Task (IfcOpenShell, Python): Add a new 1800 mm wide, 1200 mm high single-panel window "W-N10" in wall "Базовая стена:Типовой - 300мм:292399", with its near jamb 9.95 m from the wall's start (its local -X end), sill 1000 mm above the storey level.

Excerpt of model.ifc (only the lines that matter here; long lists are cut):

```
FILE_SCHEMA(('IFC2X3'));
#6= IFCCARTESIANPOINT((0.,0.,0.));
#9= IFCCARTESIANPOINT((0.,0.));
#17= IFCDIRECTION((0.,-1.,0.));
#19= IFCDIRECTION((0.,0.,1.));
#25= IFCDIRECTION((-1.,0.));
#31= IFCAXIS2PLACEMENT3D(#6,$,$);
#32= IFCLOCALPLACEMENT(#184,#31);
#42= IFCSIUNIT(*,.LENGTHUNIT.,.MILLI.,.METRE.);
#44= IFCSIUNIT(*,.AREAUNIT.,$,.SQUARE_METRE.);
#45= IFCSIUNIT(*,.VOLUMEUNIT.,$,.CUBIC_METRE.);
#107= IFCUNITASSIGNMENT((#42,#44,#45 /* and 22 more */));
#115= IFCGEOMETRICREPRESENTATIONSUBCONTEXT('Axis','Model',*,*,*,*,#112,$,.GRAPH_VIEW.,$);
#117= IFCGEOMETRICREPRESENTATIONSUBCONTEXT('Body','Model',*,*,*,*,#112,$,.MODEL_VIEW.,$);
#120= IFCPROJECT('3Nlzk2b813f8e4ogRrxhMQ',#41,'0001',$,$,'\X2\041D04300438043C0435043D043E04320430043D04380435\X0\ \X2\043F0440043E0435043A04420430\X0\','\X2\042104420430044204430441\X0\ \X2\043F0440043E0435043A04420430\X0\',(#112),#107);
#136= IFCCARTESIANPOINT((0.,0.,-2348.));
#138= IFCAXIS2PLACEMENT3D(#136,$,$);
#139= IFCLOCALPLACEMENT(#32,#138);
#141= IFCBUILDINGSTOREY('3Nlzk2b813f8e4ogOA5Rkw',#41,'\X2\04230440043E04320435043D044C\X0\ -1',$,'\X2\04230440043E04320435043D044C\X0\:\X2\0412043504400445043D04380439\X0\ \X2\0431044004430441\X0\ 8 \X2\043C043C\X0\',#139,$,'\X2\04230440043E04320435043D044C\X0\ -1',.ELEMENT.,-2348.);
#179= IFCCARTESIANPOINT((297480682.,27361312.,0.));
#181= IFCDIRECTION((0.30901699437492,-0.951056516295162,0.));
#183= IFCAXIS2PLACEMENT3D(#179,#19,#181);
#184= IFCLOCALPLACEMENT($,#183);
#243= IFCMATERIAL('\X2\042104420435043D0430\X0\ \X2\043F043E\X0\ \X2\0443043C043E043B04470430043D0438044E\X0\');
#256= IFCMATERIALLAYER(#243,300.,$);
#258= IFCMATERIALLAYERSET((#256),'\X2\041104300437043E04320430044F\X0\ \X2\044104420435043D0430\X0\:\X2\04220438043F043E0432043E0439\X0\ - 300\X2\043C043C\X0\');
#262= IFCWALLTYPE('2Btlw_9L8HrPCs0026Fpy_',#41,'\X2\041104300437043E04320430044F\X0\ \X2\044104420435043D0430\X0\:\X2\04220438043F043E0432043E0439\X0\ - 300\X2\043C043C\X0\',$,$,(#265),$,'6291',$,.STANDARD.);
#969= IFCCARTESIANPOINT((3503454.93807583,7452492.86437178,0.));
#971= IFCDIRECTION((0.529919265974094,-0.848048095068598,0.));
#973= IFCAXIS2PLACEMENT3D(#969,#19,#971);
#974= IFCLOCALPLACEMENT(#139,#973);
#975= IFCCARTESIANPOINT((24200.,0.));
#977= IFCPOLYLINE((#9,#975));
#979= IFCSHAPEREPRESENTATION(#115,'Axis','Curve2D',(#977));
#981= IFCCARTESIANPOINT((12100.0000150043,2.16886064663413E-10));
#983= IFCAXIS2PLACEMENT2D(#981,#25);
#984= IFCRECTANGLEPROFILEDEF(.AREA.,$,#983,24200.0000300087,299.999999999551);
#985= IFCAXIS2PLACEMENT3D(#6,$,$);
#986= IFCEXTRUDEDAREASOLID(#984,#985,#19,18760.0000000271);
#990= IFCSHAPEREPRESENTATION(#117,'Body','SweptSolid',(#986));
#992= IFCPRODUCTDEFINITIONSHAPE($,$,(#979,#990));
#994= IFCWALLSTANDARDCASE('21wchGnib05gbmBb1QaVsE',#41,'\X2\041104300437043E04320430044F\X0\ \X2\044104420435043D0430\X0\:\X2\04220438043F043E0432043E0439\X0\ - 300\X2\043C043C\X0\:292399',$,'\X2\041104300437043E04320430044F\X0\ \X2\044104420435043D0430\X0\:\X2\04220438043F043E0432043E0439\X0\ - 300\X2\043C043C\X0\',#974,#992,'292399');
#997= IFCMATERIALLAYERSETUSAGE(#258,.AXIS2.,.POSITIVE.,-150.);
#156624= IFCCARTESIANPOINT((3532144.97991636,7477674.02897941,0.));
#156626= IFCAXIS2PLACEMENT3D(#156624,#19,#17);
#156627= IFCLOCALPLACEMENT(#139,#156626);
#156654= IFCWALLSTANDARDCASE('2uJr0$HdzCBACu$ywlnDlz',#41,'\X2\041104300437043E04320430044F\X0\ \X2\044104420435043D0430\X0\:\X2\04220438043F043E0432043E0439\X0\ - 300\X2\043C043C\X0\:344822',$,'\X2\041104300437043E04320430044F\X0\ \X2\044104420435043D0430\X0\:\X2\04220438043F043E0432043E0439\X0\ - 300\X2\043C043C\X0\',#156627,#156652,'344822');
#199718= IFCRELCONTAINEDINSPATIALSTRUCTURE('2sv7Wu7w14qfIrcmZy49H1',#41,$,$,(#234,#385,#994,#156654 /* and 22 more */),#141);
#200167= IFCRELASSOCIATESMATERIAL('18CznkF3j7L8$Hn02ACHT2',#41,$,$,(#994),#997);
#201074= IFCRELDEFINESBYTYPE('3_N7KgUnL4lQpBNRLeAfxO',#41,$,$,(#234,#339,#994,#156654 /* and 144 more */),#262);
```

```python
import numpy as np
import ifcopenshell
import ifcopenshell.api.feature
import ifcopenshell.api.geometry
import ifcopenshell.api.root
import ifcopenshell.api.spatial
import ifcopenshell.api.type
import ifcopenshell.geom
import ifcopenshell.util.element
import ifcopenshell.util.placement
import ifcopenshell.util.representation
import ifcopenshell.util.shape
import ifcopenshell.util.unit

model = ifcopenshell.open("model.ifc")
unit_scale = ifcopenshell.util.unit.calculate_unit_scale(model)
settings = ifcopenshell.geom.settings()


def volume(element):
    """Net volume in cubic metres, openings subtracted."""
    shape = ifcopenshell.geom.create_shape(settings, element)
    return ifcopenshell.util.shape.get_volume(shape.geometry)


wall = model.by_guid("21wchGnib05gbmBb1QaVsE")
storey = ifcopenshell.util.element.get_container(wall, ifc_class="IfcBuildingStorey")
context = ifcopenshell.util.representation.get_context(model, "Model", "Body", "MODEL_VIEW")
before = volume(wall)

width, height, from_end, sill = 1.8, 1.2, 9.95, 1  # metres

# The wall runs along its own X axis, and the end named is its -X end.
wall_shape = ifcopenshell.geom.create_shape(settings, wall)
x, y, z = ifcopenshell.util.shape.get_vertices(wall_shape.geometry).T
start = x.min() + from_end
face, thickness = float(y.min()), float(y.max() - y.min())
wall_matrix = ifcopenshell.util.placement.get_local_placement(wall.ObjectPlacement)
level = ifcopenshell.util.placement.get_local_placement(storey.ObjectPlacement)[2, 3]


def in_wall(x, y):
    """Placement at x, y metres in the wall's axes, at sill height."""
    matrix = wall_matrix.copy()
    matrix[:, 3] = wall_matrix @ np.array([x / unit_scale, y / unit_scale, 0.0, 1.0])
    matrix[2, 3] = level + sill / unit_scale
    return matrix


# Opening: a box that overshoots both wall faces by 50 mm.
opening = ifcopenshell.api.root.create_entity(model, ifc_class="IfcOpeningElement")
box = ifcopenshell.api.geometry.add_wall_representation(
    model, context=context, length=width, height=height, thickness=thickness + 0.1
)
ifcopenshell.api.geometry.assign_representation(model, product=opening, representation=box)
ifcopenshell.api.geometry.edit_object_placement(model, product=opening, matrix=in_wall(start, face - 0.05), is_si=False)
ifcopenshell.api.feature.add_feature(model, feature=opening, element=wall)

window = ifcopenshell.api.root.create_entity(model, ifc_class="IfcWindow", name="W-N10")
window.OverallWidth, window.OverallHeight = width / unit_scale, height / unit_scale
body = ifcopenshell.api.geometry.add_window_representation(
    model,
    context=context,
    overall_width=window.OverallWidth,
    overall_height=window.OverallHeight,
    partition_type="SINGLE_PANEL",
)
ifcopenshell.api.geometry.assign_representation(model, product=window, representation=body)
ifcopenshell.api.spatial.assign_container(model, products=[window], relating_structure=storey)
fills = ifcopenshell.api.feature.add_filling(model, opening=opening, element=window)
fills.OwnerHistory = window.OwnerHistory  # required in IFC2X3

# IFC2X3 keeps the operation on the window style.
style = ifcopenshell.api.root.create_entity(model, ifc_class="IfcWindowStyle", name="W-N10")
style.OperationType, style.ConstructionType = "SINGLE_PANEL", "NOTDEFINED"
style.ParameterTakesPrecedence = style.Sizeable = False
ifcopenshell.api.type.assign_type(model, related_objects=[window], relating_type=style)

# Centre the window in the wall's thickness.
ifcopenshell.api.geometry.edit_object_placement(model, product=window, matrix=in_wall(start, face), is_si=False)
window_shape = ifcopenshell.geom.create_shape(settings, window)
depth = ifcopenshell.util.shape.get_vertices(window_shape.geometry)[:, 1]
offset = face + thickness / 2 - (depth.min() + depth.max()) / 2
ifcopenshell.api.geometry.edit_object_placement(model, product=window, matrix=in_wall(start, offset), is_si=False)

after = volume(wall)

print(f"wall volume {before:.3f} -> {after:.3f} m3")

model.write("model_rev.ifc")
```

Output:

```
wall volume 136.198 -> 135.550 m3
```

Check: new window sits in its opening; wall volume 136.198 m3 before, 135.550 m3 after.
